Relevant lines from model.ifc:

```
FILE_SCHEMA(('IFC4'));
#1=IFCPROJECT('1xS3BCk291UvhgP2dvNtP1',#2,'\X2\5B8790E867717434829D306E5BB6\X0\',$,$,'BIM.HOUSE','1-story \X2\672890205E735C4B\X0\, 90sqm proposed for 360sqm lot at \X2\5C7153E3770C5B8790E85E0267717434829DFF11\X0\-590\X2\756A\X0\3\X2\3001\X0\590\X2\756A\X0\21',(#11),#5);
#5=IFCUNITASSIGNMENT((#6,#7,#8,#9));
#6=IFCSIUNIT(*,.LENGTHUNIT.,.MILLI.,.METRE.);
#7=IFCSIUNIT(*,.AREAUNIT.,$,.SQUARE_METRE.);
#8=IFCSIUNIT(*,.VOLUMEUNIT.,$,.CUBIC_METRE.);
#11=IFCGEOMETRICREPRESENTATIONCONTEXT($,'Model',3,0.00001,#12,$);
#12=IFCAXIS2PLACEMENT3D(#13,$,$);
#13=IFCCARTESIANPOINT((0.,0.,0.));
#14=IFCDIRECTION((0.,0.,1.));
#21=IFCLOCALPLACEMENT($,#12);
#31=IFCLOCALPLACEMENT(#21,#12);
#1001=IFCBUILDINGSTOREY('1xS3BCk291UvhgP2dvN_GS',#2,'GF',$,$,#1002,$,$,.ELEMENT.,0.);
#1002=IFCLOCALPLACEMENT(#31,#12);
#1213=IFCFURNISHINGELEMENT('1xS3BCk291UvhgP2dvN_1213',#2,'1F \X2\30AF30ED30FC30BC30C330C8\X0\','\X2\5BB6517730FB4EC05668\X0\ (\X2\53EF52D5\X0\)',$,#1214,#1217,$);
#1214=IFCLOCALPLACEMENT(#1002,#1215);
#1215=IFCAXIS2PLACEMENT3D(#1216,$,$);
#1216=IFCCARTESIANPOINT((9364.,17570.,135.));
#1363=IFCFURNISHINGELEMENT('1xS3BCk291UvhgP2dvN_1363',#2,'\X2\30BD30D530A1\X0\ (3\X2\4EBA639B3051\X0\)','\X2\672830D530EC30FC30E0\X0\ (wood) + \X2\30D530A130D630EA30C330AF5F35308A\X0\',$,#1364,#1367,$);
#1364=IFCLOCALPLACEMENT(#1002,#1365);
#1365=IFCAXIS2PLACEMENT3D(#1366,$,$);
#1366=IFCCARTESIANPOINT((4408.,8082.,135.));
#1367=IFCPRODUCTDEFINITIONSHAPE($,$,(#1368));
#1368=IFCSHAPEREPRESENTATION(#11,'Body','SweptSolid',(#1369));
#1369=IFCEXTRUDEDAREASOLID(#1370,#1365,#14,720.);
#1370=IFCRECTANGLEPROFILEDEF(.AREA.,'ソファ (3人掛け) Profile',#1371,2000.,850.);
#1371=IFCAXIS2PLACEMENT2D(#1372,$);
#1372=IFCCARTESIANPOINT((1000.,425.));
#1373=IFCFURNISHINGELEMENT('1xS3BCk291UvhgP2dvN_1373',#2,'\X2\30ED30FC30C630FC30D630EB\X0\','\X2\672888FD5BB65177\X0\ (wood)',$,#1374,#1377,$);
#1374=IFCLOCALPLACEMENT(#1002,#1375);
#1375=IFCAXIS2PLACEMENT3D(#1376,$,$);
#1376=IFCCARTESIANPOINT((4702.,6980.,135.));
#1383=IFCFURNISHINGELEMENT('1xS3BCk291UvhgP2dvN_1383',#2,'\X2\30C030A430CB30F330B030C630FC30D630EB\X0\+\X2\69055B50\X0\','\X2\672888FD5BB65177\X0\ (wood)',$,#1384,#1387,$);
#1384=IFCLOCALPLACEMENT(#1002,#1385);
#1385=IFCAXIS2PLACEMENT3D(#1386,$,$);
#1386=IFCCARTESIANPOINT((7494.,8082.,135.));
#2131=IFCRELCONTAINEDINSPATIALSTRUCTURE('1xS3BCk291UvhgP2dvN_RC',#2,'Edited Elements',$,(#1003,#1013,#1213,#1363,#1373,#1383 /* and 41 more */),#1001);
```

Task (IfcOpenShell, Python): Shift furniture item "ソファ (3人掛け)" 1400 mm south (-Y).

```python
import ifcopenshell
import ifcopenshell.api.geometry
import ifcopenshell.util.placement
import ifcopenshell.util.unit

model = ifcopenshell.open("model.ifc")
unit_scale = ifcopenshell.util.unit.calculate_unit_scale(model)

item = model.by_guid("1xS3BCk291UvhgP2dvN_1363")
matrix = ifcopenshell.util.placement.get_local_placement(item.ObjectPlacement)
matrix[1, 3] -= 1.4 / unit_scale
ifcopenshell.api.geometry.edit_object_placement(model, product=item, matrix=matrix, is_si=False)

print(ifcopenshell.util.placement.get_local_placement(item.ObjectPlacement).round(3) + 0.0)

model.write("model_edited.ifc")
```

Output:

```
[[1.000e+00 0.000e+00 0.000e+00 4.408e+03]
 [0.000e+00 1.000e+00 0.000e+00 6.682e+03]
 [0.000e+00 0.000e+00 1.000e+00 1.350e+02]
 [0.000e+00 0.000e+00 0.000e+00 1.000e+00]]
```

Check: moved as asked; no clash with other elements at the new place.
